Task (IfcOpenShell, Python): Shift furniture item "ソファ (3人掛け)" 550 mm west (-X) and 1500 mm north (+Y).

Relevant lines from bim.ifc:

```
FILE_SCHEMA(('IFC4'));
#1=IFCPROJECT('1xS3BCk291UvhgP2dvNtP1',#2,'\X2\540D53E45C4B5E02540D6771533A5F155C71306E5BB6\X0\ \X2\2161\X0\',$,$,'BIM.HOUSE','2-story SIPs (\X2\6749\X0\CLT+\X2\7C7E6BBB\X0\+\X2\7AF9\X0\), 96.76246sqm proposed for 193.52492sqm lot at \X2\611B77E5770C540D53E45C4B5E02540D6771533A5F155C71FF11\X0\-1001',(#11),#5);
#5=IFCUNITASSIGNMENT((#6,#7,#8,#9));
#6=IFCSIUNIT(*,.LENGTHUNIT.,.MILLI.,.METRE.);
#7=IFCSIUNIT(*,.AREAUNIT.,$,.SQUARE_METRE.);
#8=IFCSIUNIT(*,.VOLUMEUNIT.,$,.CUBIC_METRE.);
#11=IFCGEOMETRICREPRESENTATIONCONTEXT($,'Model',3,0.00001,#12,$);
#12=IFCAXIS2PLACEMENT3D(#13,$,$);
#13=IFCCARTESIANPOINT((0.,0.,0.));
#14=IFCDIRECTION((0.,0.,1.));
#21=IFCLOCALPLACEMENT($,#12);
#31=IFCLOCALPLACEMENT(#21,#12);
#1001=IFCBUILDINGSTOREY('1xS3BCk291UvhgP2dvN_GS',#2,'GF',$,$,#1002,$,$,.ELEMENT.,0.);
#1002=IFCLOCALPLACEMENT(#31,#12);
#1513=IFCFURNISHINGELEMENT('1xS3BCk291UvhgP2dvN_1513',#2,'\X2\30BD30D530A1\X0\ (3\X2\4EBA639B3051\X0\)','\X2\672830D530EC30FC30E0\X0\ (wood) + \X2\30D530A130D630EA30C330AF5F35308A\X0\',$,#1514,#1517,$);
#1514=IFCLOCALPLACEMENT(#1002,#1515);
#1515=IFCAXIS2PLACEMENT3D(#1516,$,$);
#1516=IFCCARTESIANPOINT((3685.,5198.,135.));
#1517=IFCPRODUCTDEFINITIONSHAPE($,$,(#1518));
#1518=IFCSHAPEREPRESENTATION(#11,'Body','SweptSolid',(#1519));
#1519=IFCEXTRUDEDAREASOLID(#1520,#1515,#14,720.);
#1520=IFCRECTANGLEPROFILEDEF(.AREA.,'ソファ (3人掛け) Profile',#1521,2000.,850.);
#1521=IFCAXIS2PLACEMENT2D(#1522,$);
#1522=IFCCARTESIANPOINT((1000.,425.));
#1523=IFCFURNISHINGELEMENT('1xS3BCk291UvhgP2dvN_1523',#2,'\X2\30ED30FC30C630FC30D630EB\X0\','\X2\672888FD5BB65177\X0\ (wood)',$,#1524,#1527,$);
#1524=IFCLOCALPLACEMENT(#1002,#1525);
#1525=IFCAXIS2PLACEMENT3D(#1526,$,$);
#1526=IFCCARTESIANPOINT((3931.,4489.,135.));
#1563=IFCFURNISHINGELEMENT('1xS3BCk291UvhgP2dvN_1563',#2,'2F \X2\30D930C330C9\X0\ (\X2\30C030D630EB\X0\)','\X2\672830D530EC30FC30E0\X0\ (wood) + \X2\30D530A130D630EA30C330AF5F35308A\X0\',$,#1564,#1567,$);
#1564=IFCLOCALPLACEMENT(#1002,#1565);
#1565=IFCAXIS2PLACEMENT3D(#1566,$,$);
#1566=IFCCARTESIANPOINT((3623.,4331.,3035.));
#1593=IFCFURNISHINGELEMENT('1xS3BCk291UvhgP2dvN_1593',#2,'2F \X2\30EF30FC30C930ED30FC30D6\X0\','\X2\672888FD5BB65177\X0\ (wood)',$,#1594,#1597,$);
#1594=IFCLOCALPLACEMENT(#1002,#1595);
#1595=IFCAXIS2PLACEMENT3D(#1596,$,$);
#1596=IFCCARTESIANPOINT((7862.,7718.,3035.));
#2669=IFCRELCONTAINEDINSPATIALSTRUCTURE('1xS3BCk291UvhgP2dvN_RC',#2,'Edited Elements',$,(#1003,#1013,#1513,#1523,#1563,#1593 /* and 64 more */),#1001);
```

```python
import ifcopenshell
import ifcopenshell.api.geometry
import ifcopenshell.util.placement
import ifcopenshell.util.unit

model = ifcopenshell.open("bim.ifc")
unit_scale = ifcopenshell.util.unit.calculate_unit_scale(model)

item = model.by_guid("1xS3BCk291UvhgP2dvN_1513")
matrix = ifcopenshell.util.placement.get_local_placement(item.ObjectPlacement)
matrix[0, 3] -= 0.55 / unit_scale
matrix[1, 3] += 1.5 / unit_scale
ifcopenshell.api.geometry.edit_object_placement(model, product=item, matrix=matrix, is_si=False)

print(ifcopenshell.util.placement.get_local_placement(item.ObjectPlacement).round(3) + 0.0)

model.write("bim_rev.ifc")
```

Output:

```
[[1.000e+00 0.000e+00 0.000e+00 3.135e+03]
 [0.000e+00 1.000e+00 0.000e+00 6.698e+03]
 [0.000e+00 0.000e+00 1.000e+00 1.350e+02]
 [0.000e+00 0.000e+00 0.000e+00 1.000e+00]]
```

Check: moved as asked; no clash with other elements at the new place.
